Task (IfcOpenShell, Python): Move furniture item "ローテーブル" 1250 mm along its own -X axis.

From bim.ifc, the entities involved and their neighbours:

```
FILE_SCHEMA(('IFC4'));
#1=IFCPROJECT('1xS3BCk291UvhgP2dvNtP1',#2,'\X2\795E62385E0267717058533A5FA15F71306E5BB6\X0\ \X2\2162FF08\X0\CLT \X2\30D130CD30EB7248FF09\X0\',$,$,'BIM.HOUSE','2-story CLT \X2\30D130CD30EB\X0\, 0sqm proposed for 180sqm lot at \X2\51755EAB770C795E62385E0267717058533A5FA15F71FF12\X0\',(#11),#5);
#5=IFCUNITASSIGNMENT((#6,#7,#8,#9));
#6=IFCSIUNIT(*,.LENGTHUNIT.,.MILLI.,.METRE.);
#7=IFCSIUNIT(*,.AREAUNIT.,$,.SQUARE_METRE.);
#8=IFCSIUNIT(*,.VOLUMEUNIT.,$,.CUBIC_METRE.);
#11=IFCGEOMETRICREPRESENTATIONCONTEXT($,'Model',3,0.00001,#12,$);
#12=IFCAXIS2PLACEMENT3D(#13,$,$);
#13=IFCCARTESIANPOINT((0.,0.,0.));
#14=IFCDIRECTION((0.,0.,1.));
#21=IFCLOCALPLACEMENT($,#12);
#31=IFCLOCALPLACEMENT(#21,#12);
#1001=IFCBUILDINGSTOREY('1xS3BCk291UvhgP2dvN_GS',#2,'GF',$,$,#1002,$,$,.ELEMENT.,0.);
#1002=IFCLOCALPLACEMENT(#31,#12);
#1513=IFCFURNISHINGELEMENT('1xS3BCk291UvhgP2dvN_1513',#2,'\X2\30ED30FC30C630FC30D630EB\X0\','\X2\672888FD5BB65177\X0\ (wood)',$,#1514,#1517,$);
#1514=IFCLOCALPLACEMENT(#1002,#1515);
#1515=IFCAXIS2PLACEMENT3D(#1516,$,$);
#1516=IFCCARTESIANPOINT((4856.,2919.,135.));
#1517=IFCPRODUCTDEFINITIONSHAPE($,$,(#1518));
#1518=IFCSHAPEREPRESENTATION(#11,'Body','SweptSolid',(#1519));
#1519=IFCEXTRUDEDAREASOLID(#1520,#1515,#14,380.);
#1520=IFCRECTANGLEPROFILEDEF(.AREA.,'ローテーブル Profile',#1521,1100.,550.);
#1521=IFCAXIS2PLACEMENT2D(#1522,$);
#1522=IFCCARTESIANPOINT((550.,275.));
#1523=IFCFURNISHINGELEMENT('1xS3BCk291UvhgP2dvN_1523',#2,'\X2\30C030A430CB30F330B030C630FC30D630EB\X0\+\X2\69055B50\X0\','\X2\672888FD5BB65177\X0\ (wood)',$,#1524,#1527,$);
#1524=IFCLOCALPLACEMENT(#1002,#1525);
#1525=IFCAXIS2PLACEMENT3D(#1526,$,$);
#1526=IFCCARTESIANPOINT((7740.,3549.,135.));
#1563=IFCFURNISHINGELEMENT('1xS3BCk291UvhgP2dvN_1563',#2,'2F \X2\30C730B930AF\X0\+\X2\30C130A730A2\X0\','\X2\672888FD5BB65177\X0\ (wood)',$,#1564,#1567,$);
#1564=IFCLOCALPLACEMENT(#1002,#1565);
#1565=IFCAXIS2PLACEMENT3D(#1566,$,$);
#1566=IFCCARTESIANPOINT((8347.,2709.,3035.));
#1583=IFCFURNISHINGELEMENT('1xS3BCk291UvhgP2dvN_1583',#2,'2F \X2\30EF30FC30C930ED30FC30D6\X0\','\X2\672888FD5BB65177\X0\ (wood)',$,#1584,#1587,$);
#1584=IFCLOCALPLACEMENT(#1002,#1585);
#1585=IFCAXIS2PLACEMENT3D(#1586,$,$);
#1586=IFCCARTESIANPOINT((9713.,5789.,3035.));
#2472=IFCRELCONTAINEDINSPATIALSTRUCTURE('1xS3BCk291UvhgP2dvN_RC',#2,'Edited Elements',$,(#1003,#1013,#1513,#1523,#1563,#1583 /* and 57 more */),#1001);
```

```python
import ifcopenshell
import ifcopenshell.api.geometry
import ifcopenshell.util.placement

model = ifcopenshell.open("bim.ifc")

item = model.by_guid("1xS3BCk291UvhgP2dvN_1513")
matrix = ifcopenshell.util.placement.get_local_placement(item.ObjectPlacement)
matrix[:3, 3] -= matrix[:3, 0] * 1250.0
ifcopenshell.api.geometry.edit_object_placement(model, product=item, matrix=matrix, is_si=False)

print(ifcopenshell.util.placement.get_local_placement(item.ObjectPlacement).round(3) + 0.0)

model.write("bim_updated.ifc")
```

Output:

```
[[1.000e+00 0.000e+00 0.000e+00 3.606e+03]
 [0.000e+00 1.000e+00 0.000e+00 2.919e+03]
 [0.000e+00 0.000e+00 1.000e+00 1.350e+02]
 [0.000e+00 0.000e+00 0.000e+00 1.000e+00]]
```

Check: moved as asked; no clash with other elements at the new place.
